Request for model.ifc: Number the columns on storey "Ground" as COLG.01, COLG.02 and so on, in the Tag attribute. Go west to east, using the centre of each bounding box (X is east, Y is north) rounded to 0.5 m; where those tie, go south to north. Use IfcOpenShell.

First a look at what the model holds.

```python
import ifcopenshell
import ifcopenshell.util.element
import ifcopenshell.util.placement

model = ifcopenshell.open("model.ifc")
print(model.schema)
storey = next(s for s in model.by_type("IfcBuildingStorey") if s.Name == "Ground")
columns = [e for e in ifcopenshell.util.element.get_decomposition(storey) if e.is_a("IfcColumn")]
for e in sorted(columns, key=lambda e: e.id()):
    origin = ifcopenshell.util.placement.get_local_placement(e.ObjectPlacement)[:3, 3]
    print(e.id(), e.Tag, e.Name, origin.round(2) + 0.0, sep=" | ")
```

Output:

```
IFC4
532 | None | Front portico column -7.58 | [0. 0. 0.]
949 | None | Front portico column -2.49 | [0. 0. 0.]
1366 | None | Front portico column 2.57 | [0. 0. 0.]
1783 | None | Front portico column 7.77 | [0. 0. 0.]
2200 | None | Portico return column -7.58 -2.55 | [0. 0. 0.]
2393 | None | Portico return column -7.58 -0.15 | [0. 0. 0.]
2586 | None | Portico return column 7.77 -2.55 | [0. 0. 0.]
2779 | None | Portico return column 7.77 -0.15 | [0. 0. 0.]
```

```python
import ifcopenshell
import ifcopenshell.geom
import ifcopenshell.util.element
import ifcopenshell.util.shape

model = ifcopenshell.open("model.ifc")
settings = ifcopenshell.geom.settings()
settings.set("use-world-coords", True)


def centre(element):
    shape = ifcopenshell.geom.create_shape(settings, element)
    return ifcopenshell.util.shape.get_bbox_centroid(shape.geometry)


storey = next(s for s in model.by_type("IfcBuildingStorey") if s.Name == "Ground")
columns = [e for e in ifcopenshell.util.element.get_decomposition(storey) if e.is_a("IfcColumn")]

# Insertion points can sit at a corner or the storey origin, so sort by the geometry (in metres).
centres = {e: centre(e) for e in columns}
columns.sort(key=lambda e: (round(centres[e][0] / 0.5), centres[e][1]))

for i, e in enumerate(columns, start=1):
    number = f"COLG.{i:02d}"
    e.Tag = number
    print(e.id(), number)

model.write("model_updated.ifc")
```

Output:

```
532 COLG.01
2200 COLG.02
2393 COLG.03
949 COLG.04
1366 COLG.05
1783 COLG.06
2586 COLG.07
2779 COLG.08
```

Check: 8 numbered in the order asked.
